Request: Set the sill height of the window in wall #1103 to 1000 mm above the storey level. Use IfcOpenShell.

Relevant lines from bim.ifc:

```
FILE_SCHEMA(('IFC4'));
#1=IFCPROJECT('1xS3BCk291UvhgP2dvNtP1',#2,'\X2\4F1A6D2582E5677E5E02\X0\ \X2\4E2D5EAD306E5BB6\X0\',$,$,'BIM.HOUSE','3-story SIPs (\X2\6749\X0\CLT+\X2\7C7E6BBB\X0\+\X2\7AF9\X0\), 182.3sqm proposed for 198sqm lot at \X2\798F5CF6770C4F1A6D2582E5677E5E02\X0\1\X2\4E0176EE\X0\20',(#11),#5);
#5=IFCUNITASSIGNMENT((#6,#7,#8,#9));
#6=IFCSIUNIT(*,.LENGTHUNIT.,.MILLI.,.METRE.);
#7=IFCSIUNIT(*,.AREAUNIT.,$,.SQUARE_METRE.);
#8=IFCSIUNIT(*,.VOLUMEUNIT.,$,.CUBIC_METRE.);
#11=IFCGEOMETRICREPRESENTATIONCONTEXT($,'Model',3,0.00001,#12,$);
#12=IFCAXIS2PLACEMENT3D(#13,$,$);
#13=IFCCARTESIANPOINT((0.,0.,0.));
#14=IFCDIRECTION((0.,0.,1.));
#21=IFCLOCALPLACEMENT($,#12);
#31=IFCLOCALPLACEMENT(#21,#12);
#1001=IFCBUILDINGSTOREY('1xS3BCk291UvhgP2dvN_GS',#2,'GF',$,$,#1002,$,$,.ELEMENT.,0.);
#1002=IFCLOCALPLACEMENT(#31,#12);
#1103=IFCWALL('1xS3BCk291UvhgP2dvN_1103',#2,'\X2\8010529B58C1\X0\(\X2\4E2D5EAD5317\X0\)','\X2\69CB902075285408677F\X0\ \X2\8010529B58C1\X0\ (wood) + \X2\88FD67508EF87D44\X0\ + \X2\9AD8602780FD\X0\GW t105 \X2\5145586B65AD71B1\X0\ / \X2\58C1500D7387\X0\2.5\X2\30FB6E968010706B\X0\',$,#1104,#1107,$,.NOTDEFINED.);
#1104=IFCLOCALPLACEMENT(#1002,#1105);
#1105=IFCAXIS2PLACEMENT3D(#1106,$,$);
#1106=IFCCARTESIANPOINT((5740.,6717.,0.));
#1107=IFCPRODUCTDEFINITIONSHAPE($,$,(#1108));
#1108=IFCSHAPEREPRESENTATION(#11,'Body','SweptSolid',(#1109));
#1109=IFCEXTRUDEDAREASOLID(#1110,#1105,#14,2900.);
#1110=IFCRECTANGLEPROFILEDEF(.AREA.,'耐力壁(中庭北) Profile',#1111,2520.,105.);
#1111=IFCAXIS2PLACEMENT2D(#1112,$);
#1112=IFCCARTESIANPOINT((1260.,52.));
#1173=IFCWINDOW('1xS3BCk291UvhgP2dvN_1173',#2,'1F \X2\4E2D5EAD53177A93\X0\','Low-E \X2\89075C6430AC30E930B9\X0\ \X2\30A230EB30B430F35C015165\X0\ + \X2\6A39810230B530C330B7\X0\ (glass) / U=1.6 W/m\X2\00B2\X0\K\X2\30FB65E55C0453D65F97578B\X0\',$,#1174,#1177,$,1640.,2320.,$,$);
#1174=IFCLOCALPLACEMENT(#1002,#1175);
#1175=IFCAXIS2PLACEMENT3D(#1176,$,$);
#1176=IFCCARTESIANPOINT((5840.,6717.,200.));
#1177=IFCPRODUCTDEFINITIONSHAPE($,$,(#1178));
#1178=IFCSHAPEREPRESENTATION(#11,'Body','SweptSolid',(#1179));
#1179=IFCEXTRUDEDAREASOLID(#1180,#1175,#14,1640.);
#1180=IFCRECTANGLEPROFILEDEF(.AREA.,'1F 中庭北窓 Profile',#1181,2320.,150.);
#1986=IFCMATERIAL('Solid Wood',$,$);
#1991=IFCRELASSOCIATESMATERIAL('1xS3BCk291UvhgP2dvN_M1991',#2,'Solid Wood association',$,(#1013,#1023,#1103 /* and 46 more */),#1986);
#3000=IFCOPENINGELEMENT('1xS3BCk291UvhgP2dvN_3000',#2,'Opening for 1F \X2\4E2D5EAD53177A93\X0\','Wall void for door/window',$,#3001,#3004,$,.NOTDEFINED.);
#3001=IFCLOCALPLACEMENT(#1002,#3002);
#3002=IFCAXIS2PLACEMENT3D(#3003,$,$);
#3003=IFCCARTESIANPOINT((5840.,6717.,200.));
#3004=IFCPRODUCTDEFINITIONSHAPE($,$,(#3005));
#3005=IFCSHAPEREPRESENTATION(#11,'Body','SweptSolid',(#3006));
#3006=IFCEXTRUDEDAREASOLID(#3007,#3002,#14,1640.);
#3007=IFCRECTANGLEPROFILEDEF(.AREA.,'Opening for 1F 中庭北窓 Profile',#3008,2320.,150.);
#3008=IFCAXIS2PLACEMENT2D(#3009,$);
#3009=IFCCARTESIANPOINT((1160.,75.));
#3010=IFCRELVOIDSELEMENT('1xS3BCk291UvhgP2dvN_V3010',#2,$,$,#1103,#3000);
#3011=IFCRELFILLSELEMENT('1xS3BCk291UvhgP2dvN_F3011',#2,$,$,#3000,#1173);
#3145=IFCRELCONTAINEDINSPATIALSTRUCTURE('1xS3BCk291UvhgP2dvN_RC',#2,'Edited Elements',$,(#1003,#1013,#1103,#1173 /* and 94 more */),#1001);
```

```python
import numpy as np
import ifcopenshell
import ifcopenshell.api.geometry
import ifcopenshell.geom
import ifcopenshell.util.element
import ifcopenshell.util.placement
import ifcopenshell.util.shape
import ifcopenshell.util.unit

model = ifcopenshell.open("bim.ifc")
unit_scale = ifcopenshell.util.unit.calculate_unit_scale(model)

window = model.by_guid("1xS3BCk291UvhgP2dvN_1173")
opening = window.FillsVoids[0].RelatingOpeningElement
storey = ifcopenshell.util.element.get_container(window, ifc_class="IfcBuildingStorey")
level = ifcopenshell.util.placement.get_local_placement(storey.ObjectPlacement)[2, 3]

# The opening's origin need not be at the sill, so measure its lowest point.
shape = ifcopenshell.geom.create_shape(ifcopenshell.geom.settings(), opening)
bottom = ifcopenshell.util.shape.get_shape_bottom_elevation(shape, shape.geometry) / unit_scale
dz = level + 1000.0 - bottom

shift = np.array([0.0, 0.0, dz])
# The window is not placed relative to its opening, so move both.
for product in (opening, window):
    matrix = ifcopenshell.util.placement.get_local_placement(product.ObjectPlacement)
    matrix[:3, 3] += shift
    ifcopenshell.api.geometry.edit_object_placement(model, product=product, matrix=matrix, is_si=False)

print(f"moved by {dz * unit_scale:+.3f} m")

model.write("bim_updated.ifc")
```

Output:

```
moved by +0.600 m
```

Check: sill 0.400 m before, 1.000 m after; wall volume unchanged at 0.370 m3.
